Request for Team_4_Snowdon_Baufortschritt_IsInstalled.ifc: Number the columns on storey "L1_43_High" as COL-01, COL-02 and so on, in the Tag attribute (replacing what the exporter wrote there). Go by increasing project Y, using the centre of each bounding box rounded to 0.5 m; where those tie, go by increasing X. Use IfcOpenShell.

First a look at what the model holds.

```python
import ifcopenshell
import ifcopenshell.util.element
import ifcopenshell.util.placement

model = ifcopenshell.open("Team_4_Snowdon_Baufortschritt_IsInstalled.ifc")
print(model.schema)
storey = next(s for s in model.by_type("IfcBuildingStorey") if s.Name == "L1_43_High")
columns = [e for e in ifcopenshell.util.element.get_decomposition(storey) if e.is_a("IfcColumn")]
for e in sorted(columns, key=lambda e: e.id()):
    origin = ifcopenshell.util.placement.get_local_placement(e.ObjectPlacement)[:3, 3]
    print(e.id(), e.Tag, e.Name, origin.round(2) + 0.0, sep=" | ")
```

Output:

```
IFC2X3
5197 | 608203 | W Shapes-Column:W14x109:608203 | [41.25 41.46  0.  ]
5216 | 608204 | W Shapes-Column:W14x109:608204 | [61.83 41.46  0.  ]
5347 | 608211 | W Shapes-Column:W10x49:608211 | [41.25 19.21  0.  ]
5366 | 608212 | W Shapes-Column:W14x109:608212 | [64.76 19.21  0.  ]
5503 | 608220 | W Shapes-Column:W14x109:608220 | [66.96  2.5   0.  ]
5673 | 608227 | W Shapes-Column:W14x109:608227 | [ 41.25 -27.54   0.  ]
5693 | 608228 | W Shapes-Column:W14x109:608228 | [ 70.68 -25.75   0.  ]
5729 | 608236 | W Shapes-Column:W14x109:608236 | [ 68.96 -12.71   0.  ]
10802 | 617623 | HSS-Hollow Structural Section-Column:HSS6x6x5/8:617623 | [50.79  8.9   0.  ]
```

```python
import ifcopenshell
import ifcopenshell.geom
import ifcopenshell.util.element
import ifcopenshell.util.shape

model = ifcopenshell.open("Team_4_Snowdon_Baufortschritt_IsInstalled.ifc")
settings = ifcopenshell.geom.settings()
settings.set("use-world-coords", True)


def centre(element):
    shape = ifcopenshell.geom.create_shape(settings, element)
    return ifcopenshell.util.shape.get_bbox_centroid(shape.geometry)


storey = next(s for s in model.by_type("IfcBuildingStorey") if s.Name == "L1_43_High")
columns = [e for e in ifcopenshell.util.element.get_decomposition(storey) if e.is_a("IfcColumn")]

# Insertion points can sit at a corner or the storey origin, so sort by the geometry (in metres).
centres = {e: centre(e) for e in columns}
columns.sort(key=lambda e: (round(centres[e][1] / 0.5), centres[e][0]))

for i, e in enumerate(columns, start=1):
    number = f"COL-{i:02d}"
    e.Tag = number
    print(e.id(), number)

model.write("Team_4_Snowdon_Baufortschritt_IsInstalled-out.ifc")
```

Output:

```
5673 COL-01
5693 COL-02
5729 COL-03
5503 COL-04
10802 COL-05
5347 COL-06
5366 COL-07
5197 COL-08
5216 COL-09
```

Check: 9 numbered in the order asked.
